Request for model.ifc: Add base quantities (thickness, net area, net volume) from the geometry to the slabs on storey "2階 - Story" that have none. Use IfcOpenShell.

First a look at what the model holds.

```python
import ifcopenshell
import ifcopenshell.util.element
import ifcopenshell.util.unit

model = ifcopenshell.open("model.ifc")
print(model.schema)
for unit_type in ("LENGTHUNIT", "AREAUNIT", "VOLUMEUNIT"):
    print(unit_type, ifcopenshell.util.unit.calculate_unit_scale(model, unit_type))
storey = next(s for s in model.by_type("IfcBuildingStorey") if s.Name == "2階 - Story")
slabs = [e for e in ifcopenshell.util.element.get_decomposition(storey) if e.is_a("IfcSlab")]
for e in sorted(slabs, key=lambda e: e.id()):
    print(e.id(), e.is_a(), e.Name, list(ifcopenshell.util.element.get_psets(e, qtos_only=True)), sep=" | ")
```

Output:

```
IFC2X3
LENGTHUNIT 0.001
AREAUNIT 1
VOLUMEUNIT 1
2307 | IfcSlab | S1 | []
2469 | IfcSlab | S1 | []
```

```python
import ifcopenshell
import ifcopenshell.api.pset
import ifcopenshell.geom
import ifcopenshell.util.element
import ifcopenshell.util.shape
import ifcopenshell.util.unit

model = ifcopenshell.open("model.ifc")
unit_scale = ifcopenshell.util.unit.calculate_unit_scale(model)
area_scale = ifcopenshell.util.unit.calculate_unit_scale(model, "AREAUNIT")
volume_scale = ifcopenshell.util.unit.calculate_unit_scale(model, "VOLUMEUNIT")
settings = ifcopenshell.geom.settings()

storey = next(s for s in model.by_type("IfcBuildingStorey") if s.Name == "2階 - Story")
slabs = [e for e in ifcopenshell.util.element.get_decomposition(storey) if e.is_a("IfcSlab")]

for e in sorted(slabs, key=lambda e: e.id()):
    if ifcopenshell.util.element.get_psets(e, qtos_only=True, should_inherit=False):
        continue
    # Geometry comes back in metres, in the element's own axes.
    shape = ifcopenshell.geom.create_shape(settings, e)
    values = {
        "Width": ifcopenshell.util.shape.get_z(shape.geometry) / unit_scale,
        "NetArea": ifcopenshell.util.shape.get_footprint_area(shape.geometry) / area_scale,
        "NetVolume": ifcopenshell.util.shape.get_volume(shape.geometry) / volume_scale,
    }
    qto = ifcopenshell.api.pset.add_qto(model, product=e, name="BaseQuantities")
    ifcopenshell.api.pset.edit_qto(model, qto=qto, properties=values)
    print(e.id(), {k: round(v, 3) for k, v in values.items()})

model.write("model-out.ifc")
```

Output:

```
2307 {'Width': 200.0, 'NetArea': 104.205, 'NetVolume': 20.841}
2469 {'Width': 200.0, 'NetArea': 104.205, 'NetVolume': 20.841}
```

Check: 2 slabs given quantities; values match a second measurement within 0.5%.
